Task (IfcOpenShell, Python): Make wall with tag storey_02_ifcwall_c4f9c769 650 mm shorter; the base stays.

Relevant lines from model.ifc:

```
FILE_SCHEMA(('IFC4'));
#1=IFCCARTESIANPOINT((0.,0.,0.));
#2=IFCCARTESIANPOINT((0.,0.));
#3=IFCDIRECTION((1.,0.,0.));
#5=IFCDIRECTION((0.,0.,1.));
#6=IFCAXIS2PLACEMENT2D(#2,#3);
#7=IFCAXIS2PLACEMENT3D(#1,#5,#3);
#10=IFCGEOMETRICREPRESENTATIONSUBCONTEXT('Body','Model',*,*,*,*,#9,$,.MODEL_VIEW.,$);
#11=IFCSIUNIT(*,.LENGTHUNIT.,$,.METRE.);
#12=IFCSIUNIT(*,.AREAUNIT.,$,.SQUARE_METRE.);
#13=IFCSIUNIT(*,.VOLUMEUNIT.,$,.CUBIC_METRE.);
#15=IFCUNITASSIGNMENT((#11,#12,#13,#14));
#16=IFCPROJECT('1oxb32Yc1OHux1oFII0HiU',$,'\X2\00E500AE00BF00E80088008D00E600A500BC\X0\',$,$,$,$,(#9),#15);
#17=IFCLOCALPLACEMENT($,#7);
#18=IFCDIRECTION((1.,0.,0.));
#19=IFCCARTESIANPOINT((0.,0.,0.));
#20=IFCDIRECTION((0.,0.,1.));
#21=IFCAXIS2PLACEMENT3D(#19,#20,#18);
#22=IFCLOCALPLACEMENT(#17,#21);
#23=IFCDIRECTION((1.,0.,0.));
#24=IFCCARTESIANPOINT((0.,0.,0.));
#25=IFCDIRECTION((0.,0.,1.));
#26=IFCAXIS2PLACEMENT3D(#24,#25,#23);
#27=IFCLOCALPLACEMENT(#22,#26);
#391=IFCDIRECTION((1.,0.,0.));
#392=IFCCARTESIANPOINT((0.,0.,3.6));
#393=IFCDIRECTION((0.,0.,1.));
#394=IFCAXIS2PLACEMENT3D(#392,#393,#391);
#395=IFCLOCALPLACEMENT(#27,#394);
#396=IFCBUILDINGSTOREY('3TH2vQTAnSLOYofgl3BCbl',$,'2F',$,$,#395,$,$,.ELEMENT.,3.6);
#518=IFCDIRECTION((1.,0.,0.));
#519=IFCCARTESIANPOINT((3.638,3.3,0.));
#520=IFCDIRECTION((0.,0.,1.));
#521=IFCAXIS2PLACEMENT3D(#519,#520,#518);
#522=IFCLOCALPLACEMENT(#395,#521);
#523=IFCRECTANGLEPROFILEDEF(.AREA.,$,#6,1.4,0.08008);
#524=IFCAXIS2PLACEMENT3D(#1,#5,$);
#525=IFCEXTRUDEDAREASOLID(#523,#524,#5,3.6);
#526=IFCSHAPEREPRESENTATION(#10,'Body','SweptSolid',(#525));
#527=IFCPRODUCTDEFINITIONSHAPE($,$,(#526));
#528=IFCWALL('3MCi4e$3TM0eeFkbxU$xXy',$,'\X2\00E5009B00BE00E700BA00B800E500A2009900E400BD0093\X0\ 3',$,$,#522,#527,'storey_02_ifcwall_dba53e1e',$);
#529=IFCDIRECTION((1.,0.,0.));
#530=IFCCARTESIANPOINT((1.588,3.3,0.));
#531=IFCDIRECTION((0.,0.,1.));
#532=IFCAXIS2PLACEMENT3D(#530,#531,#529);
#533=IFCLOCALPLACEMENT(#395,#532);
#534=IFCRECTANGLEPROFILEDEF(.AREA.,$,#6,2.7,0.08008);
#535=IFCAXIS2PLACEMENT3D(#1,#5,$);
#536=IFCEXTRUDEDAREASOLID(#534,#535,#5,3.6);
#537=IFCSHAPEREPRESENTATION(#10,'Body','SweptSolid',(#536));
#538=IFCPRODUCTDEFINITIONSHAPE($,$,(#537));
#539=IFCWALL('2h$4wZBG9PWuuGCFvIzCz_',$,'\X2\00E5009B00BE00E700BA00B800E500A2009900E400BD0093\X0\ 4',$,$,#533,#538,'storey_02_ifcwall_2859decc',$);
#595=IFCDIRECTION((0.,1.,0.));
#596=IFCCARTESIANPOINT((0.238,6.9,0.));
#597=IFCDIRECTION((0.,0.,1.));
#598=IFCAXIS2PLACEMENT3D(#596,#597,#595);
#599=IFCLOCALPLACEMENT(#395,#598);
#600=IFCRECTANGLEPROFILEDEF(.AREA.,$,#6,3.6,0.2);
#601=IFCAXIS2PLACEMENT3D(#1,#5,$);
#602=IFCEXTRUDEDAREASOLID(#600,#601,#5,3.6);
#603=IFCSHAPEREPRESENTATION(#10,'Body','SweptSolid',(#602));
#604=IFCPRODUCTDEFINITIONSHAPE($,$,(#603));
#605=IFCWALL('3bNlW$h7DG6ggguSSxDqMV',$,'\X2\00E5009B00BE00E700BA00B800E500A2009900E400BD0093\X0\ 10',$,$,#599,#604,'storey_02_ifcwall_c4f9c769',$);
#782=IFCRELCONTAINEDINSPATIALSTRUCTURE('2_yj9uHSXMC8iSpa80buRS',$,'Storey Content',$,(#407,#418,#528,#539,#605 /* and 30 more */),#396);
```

```python
import ifcopenshell
import ifcopenshell.geom
import ifcopenshell.util.representation
import ifcopenshell.util.shape
import ifcopenshell.util.unit

model = ifcopenshell.open("model.ifc")
unit_scale = ifcopenshell.util.unit.calculate_unit_scale(model)
settings = ifcopenshell.geom.settings()


def volume(element):
    """Net volume in cubic metres, openings subtracted."""
    shape = ifcopenshell.geom.create_shape(settings, element)
    return ifcopenshell.util.shape.get_volume(shape.geometry)


wall = model.by_guid("3bNlW$h7DG6ggguSSxDqMV")
before = volume(wall)

body = ifcopenshell.util.representation.get_representation(wall, "Model", "Body")
solid = body.Items[0]
old_height = solid.Depth
solid.Depth -= 0.65 / unit_scale
after = volume(wall)

print(f"height {old_height:g} -> {solid.Depth:g}, volume {before:.3f} -> {after:.3f} m3")

model.write("model_updated.ifc")
```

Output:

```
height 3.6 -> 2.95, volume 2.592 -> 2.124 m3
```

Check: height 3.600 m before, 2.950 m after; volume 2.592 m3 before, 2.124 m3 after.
